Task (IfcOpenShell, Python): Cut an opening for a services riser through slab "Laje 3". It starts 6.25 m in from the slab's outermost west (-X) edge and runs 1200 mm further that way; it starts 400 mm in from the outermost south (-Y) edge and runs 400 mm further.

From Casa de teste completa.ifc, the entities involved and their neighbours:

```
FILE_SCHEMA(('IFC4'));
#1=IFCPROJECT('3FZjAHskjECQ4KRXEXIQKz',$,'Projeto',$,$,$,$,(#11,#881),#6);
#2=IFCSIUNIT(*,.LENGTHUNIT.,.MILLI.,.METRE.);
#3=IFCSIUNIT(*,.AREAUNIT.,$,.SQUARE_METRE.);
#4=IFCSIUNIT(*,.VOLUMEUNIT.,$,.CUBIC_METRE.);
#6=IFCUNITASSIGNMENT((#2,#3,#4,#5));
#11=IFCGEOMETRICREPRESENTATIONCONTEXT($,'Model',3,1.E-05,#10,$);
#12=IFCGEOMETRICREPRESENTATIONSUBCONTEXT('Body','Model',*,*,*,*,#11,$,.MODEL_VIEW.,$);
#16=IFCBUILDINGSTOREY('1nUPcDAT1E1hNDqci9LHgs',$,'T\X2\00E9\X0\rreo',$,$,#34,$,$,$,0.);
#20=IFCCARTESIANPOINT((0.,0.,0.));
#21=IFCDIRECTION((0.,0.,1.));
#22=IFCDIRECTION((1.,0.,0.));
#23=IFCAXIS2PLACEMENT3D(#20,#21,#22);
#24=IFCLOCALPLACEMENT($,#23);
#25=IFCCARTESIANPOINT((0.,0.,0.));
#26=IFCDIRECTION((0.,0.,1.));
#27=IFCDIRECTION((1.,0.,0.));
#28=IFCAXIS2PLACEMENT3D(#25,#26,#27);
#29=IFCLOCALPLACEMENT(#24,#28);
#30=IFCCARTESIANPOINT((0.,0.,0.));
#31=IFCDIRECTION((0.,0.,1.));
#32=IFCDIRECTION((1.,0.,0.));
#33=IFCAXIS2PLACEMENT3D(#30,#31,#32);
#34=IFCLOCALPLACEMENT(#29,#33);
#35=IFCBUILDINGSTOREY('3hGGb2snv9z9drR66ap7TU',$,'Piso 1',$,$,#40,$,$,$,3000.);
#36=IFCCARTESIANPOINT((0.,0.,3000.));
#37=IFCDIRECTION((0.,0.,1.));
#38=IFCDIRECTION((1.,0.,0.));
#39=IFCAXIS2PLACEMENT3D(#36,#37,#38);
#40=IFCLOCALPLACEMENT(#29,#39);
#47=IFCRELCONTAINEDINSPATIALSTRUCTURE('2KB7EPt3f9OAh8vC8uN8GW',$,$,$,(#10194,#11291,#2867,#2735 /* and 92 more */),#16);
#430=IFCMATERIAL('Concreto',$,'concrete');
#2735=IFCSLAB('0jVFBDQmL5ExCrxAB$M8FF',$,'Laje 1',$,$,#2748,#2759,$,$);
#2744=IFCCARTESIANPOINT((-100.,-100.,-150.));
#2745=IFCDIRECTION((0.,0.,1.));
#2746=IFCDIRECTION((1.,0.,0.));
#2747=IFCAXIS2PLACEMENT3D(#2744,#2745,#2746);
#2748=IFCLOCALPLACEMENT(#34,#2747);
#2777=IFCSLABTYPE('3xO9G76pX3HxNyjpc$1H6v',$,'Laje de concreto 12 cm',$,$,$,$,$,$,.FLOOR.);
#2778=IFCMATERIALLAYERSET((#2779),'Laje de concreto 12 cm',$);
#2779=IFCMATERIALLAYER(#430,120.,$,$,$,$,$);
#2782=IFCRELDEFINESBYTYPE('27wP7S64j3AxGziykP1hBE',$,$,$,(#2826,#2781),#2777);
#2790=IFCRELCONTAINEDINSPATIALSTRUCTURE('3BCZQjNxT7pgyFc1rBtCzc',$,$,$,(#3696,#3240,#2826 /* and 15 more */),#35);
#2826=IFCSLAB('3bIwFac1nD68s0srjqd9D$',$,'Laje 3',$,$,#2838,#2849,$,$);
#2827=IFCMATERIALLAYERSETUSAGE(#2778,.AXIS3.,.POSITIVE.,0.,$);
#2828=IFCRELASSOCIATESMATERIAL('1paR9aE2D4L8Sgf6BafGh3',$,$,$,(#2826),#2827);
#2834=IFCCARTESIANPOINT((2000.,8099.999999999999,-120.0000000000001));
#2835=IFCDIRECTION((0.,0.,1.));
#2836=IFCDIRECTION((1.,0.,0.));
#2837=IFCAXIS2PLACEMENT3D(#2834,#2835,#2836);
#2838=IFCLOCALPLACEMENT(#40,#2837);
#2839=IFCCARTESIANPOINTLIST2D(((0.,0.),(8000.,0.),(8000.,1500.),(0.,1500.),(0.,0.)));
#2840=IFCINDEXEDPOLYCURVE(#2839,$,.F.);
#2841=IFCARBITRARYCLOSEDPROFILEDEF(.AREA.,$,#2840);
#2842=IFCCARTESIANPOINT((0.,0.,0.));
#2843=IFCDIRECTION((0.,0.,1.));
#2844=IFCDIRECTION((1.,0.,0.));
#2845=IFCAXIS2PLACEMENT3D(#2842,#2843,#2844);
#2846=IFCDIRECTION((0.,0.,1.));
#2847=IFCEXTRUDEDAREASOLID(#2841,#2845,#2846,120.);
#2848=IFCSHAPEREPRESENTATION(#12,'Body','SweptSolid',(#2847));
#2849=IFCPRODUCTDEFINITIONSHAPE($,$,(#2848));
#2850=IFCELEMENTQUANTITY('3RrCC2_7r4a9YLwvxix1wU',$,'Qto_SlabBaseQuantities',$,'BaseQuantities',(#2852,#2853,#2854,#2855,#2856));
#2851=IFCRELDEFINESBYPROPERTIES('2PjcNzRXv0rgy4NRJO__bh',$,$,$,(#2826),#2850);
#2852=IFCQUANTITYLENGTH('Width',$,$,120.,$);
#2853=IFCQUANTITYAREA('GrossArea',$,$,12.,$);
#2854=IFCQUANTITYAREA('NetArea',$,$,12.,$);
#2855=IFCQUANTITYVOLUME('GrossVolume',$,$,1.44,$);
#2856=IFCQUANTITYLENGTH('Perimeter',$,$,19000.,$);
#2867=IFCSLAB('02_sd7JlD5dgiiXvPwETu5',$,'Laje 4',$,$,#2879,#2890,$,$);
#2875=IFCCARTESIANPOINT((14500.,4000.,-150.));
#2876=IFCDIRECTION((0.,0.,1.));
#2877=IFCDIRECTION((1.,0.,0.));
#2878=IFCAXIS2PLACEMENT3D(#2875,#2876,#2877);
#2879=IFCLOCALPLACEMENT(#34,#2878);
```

```python
import numpy as np
import ifcopenshell
import ifcopenshell.api.feature
import ifcopenshell.api.geometry
import ifcopenshell.api.pset
import ifcopenshell.api.root
import ifcopenshell.geom
import ifcopenshell.util.element
import ifcopenshell.util.placement
import ifcopenshell.util.representation
import ifcopenshell.util.shape
import ifcopenshell.util.unit

model = ifcopenshell.open("Casa de teste completa.ifc")
unit_scale = ifcopenshell.util.unit.calculate_unit_scale(model)
area_scale = ifcopenshell.util.unit.calculate_unit_scale(model, "AREAUNIT")
settings = ifcopenshell.geom.settings()


def volume(element):
    """Net volume in cubic metres, openings subtracted."""
    shape = ifcopenshell.geom.create_shape(settings, element)
    return ifcopenshell.util.shape.get_volume(shape.geometry)


slab = model.by_guid("3bIwFac1nD68s0srjqd9D$")
before = volume(slab)

# Extent in the slab's own axes, in metres. The edges named are its -X and -Y sides.
slab_shape = ifcopenshell.geom.create_shape(settings, slab)
vertices = ifcopenshell.util.shape.get_vertices(slab_shape.geometry)
x_min, y_min, bottom = vertices.min(axis=0)
top = vertices[:, 2].max()

opening = ifcopenshell.api.root.create_entity(model, ifc_class="IfcOpeningElement", name="Services riser opening", predefined_type="OPENING")
context = ifcopenshell.util.representation.get_context(model, "Model", "Body", "MODEL_VIEW")
width, depth = 1.2, 0.4
outline = [(0.0, 0.0), (width, 0.0), (width, depth), (0.0, depth), (0.0, 0.0)]
# Overshoot both faces by 50 mm so the cut is clean.
shape = ifcopenshell.api.geometry.add_slab_representation(
    model, context=context, depth=top - bottom + 0.1, polyline=outline
)
ifcopenshell.api.geometry.assign_representation(model, product=opening, representation=shape)

matrix = ifcopenshell.util.placement.get_local_placement(slab.ObjectPlacement)
matrix[:, 3] = matrix @ np.append(np.array([x_min + 6.25, y_min + 0.4, bottom - 0.05]) / unit_scale, 1.0)
ifcopenshell.api.geometry.edit_object_placement(model, product=opening, matrix=matrix, is_si=False)
ifcopenshell.api.feature.add_feature(model, feature=opening, element=slab)

after = volume(slab)

# Update the slab's stored quantities.
qto = model.by_id(ifcopenshell.util.element.get_pset(slab, "Qto_SlabBaseQuantities", should_inherit=False)["id"])
ifcopenshell.api.pset.edit_qto(model, qto=qto, properties={"NetArea": after / (top - bottom) / area_scale})

print(f"slab volume {before:.3f} -> {after:.3f} m3")

model.write("Casa de teste completa_rev.ifc")
```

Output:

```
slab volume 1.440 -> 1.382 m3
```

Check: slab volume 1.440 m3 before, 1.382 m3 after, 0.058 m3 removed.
